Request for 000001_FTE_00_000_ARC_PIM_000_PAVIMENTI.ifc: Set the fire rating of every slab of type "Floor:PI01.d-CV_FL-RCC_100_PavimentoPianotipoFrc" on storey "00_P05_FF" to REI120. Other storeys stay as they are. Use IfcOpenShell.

First a look at what the model holds.

```python
import ifcopenshell
import ifcopenshell.util.element

model = ifcopenshell.open("000001_FTE_00_000_ARC_PIM_000_PAVIMENTI.ifc")
print(model.schema)
storey = next(s for s in model.by_type("IfcBuildingStorey") if s.Name == "00_P05_FF")
slabs = [e for e in ifcopenshell.util.element.get_decomposition(storey) if e.is_a("IfcSlab")]
seen = {}
for e in slabs:
    element_type = ifcopenshell.util.element.get_type(e)
    key = (element_type.Name if element_type != e and element_type else None, ifcopenshell.util.element.get_pset(e, "Pset_SlabCommon", "FireRating"))
    seen[key] = seen.get(key, 0) + 1
for (name, value), count in sorted(seen.items(), key=str):
    print(count, "x", name, "|", value)
```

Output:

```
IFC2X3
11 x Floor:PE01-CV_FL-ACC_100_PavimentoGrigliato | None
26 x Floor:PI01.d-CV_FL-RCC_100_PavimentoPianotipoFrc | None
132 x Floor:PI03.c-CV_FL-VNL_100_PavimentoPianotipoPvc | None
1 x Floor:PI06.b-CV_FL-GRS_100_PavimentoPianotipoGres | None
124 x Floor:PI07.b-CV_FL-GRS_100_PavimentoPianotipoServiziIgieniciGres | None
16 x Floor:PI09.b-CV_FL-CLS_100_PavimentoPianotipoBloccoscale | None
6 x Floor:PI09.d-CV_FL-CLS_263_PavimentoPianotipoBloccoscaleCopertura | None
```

```python
import ifcopenshell
import ifcopenshell.api.pset
import ifcopenshell.util.element

model = ifcopenshell.open("000001_FTE_00_000_ARC_PIM_000_PAVIMENTI.ifc")

storey = next(s for s in model.by_type("IfcBuildingStorey") if s.Name == "00_P05_FF")
slabs = [e for e in ifcopenshell.util.element.get_decomposition(storey) if e.is_a("IfcSlab")]

count = 0
for e in slabs:
    element_type = ifcopenshell.util.element.get_type(e)
    if element_type in (None, e) or element_type.Name != "Floor:PI01.d-CV_FL-RCC_100_PavimentoPianotipoFrc":
        continue
    # add_pset returns the element's existing set when there is one.
    pset = ifcopenshell.api.pset.add_pset(model, product=e, name="Pset_SlabCommon")
    ifcopenshell.api.pset.edit_pset(model, pset=pset, properties={"FireRating": "REI120"})
    count += 1

print(count, "slabs updated")

model.write("000001_FTE_00_000_ARC_PIM_000_PAVIMENTI-out.ifc")
```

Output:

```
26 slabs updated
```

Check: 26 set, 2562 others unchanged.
